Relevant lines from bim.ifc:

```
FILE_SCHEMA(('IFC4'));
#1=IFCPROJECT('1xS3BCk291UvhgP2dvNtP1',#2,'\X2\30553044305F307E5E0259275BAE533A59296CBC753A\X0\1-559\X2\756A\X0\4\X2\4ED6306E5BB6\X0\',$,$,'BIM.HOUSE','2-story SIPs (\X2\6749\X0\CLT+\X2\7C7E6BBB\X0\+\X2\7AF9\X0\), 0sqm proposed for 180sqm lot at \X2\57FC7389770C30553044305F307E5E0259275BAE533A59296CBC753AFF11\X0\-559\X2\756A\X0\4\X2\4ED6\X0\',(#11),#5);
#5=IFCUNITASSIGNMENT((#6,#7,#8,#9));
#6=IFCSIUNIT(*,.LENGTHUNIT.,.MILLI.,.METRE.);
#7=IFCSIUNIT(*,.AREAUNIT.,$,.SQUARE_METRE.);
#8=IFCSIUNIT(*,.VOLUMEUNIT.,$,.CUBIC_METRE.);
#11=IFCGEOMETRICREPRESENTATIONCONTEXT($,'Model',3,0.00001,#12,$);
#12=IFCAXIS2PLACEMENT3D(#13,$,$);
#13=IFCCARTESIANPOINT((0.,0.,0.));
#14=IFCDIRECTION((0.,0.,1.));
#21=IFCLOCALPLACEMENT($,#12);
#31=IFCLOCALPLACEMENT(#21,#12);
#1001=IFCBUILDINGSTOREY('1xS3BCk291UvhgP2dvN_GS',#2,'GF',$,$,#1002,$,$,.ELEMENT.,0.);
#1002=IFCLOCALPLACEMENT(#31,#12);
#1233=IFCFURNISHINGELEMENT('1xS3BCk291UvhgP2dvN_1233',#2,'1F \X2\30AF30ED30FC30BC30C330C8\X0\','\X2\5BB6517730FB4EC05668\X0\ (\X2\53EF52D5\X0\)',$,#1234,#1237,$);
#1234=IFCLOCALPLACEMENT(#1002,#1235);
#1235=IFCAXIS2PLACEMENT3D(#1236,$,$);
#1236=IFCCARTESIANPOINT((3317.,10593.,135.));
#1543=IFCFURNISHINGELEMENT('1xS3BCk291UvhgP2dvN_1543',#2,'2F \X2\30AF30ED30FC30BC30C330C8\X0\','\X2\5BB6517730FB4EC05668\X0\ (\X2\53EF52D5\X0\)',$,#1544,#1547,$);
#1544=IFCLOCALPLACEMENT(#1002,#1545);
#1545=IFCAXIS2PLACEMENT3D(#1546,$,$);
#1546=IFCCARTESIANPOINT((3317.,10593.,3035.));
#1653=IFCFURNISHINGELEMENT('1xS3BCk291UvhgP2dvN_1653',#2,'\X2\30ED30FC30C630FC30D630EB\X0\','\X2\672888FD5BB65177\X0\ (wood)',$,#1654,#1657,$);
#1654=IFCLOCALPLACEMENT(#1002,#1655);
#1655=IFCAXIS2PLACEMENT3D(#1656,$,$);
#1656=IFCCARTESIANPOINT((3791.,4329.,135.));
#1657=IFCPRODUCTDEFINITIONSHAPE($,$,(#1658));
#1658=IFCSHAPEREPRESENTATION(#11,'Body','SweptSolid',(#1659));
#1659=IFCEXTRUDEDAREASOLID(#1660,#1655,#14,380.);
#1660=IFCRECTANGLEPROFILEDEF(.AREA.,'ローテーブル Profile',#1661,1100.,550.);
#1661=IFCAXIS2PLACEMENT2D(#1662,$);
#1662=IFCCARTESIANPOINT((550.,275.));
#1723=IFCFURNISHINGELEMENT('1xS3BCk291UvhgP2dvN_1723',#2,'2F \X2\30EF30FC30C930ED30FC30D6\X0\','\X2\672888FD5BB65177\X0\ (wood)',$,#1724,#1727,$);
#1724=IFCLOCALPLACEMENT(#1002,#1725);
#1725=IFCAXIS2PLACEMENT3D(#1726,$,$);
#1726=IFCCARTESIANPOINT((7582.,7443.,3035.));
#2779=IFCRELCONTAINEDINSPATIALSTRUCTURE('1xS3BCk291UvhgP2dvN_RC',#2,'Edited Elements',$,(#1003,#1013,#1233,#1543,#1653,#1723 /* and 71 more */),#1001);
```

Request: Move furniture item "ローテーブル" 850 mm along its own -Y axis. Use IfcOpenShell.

```python
import ifcopenshell
import ifcopenshell.api.geometry
import ifcopenshell.util.placement
import ifcopenshell.util.unit

model = ifcopenshell.open("bim.ifc")
unit_scale = ifcopenshell.util.unit.calculate_unit_scale(model)

item = model.by_id(1653)
matrix = ifcopenshell.util.placement.get_local_placement(item.ObjectPlacement)
matrix[:3, 3] -= matrix[:3, 1] * 0.85 / unit_scale
ifcopenshell.api.geometry.edit_object_placement(model, product=item, matrix=matrix, is_si=False)

print(ifcopenshell.util.placement.get_local_placement(item.ObjectPlacement).round(3) + 0.0)

model.write("bim-out.ifc")
```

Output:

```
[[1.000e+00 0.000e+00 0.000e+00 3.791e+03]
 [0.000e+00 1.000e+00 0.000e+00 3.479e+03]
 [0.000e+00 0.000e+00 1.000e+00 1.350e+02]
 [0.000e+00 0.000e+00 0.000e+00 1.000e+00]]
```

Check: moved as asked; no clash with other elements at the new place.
